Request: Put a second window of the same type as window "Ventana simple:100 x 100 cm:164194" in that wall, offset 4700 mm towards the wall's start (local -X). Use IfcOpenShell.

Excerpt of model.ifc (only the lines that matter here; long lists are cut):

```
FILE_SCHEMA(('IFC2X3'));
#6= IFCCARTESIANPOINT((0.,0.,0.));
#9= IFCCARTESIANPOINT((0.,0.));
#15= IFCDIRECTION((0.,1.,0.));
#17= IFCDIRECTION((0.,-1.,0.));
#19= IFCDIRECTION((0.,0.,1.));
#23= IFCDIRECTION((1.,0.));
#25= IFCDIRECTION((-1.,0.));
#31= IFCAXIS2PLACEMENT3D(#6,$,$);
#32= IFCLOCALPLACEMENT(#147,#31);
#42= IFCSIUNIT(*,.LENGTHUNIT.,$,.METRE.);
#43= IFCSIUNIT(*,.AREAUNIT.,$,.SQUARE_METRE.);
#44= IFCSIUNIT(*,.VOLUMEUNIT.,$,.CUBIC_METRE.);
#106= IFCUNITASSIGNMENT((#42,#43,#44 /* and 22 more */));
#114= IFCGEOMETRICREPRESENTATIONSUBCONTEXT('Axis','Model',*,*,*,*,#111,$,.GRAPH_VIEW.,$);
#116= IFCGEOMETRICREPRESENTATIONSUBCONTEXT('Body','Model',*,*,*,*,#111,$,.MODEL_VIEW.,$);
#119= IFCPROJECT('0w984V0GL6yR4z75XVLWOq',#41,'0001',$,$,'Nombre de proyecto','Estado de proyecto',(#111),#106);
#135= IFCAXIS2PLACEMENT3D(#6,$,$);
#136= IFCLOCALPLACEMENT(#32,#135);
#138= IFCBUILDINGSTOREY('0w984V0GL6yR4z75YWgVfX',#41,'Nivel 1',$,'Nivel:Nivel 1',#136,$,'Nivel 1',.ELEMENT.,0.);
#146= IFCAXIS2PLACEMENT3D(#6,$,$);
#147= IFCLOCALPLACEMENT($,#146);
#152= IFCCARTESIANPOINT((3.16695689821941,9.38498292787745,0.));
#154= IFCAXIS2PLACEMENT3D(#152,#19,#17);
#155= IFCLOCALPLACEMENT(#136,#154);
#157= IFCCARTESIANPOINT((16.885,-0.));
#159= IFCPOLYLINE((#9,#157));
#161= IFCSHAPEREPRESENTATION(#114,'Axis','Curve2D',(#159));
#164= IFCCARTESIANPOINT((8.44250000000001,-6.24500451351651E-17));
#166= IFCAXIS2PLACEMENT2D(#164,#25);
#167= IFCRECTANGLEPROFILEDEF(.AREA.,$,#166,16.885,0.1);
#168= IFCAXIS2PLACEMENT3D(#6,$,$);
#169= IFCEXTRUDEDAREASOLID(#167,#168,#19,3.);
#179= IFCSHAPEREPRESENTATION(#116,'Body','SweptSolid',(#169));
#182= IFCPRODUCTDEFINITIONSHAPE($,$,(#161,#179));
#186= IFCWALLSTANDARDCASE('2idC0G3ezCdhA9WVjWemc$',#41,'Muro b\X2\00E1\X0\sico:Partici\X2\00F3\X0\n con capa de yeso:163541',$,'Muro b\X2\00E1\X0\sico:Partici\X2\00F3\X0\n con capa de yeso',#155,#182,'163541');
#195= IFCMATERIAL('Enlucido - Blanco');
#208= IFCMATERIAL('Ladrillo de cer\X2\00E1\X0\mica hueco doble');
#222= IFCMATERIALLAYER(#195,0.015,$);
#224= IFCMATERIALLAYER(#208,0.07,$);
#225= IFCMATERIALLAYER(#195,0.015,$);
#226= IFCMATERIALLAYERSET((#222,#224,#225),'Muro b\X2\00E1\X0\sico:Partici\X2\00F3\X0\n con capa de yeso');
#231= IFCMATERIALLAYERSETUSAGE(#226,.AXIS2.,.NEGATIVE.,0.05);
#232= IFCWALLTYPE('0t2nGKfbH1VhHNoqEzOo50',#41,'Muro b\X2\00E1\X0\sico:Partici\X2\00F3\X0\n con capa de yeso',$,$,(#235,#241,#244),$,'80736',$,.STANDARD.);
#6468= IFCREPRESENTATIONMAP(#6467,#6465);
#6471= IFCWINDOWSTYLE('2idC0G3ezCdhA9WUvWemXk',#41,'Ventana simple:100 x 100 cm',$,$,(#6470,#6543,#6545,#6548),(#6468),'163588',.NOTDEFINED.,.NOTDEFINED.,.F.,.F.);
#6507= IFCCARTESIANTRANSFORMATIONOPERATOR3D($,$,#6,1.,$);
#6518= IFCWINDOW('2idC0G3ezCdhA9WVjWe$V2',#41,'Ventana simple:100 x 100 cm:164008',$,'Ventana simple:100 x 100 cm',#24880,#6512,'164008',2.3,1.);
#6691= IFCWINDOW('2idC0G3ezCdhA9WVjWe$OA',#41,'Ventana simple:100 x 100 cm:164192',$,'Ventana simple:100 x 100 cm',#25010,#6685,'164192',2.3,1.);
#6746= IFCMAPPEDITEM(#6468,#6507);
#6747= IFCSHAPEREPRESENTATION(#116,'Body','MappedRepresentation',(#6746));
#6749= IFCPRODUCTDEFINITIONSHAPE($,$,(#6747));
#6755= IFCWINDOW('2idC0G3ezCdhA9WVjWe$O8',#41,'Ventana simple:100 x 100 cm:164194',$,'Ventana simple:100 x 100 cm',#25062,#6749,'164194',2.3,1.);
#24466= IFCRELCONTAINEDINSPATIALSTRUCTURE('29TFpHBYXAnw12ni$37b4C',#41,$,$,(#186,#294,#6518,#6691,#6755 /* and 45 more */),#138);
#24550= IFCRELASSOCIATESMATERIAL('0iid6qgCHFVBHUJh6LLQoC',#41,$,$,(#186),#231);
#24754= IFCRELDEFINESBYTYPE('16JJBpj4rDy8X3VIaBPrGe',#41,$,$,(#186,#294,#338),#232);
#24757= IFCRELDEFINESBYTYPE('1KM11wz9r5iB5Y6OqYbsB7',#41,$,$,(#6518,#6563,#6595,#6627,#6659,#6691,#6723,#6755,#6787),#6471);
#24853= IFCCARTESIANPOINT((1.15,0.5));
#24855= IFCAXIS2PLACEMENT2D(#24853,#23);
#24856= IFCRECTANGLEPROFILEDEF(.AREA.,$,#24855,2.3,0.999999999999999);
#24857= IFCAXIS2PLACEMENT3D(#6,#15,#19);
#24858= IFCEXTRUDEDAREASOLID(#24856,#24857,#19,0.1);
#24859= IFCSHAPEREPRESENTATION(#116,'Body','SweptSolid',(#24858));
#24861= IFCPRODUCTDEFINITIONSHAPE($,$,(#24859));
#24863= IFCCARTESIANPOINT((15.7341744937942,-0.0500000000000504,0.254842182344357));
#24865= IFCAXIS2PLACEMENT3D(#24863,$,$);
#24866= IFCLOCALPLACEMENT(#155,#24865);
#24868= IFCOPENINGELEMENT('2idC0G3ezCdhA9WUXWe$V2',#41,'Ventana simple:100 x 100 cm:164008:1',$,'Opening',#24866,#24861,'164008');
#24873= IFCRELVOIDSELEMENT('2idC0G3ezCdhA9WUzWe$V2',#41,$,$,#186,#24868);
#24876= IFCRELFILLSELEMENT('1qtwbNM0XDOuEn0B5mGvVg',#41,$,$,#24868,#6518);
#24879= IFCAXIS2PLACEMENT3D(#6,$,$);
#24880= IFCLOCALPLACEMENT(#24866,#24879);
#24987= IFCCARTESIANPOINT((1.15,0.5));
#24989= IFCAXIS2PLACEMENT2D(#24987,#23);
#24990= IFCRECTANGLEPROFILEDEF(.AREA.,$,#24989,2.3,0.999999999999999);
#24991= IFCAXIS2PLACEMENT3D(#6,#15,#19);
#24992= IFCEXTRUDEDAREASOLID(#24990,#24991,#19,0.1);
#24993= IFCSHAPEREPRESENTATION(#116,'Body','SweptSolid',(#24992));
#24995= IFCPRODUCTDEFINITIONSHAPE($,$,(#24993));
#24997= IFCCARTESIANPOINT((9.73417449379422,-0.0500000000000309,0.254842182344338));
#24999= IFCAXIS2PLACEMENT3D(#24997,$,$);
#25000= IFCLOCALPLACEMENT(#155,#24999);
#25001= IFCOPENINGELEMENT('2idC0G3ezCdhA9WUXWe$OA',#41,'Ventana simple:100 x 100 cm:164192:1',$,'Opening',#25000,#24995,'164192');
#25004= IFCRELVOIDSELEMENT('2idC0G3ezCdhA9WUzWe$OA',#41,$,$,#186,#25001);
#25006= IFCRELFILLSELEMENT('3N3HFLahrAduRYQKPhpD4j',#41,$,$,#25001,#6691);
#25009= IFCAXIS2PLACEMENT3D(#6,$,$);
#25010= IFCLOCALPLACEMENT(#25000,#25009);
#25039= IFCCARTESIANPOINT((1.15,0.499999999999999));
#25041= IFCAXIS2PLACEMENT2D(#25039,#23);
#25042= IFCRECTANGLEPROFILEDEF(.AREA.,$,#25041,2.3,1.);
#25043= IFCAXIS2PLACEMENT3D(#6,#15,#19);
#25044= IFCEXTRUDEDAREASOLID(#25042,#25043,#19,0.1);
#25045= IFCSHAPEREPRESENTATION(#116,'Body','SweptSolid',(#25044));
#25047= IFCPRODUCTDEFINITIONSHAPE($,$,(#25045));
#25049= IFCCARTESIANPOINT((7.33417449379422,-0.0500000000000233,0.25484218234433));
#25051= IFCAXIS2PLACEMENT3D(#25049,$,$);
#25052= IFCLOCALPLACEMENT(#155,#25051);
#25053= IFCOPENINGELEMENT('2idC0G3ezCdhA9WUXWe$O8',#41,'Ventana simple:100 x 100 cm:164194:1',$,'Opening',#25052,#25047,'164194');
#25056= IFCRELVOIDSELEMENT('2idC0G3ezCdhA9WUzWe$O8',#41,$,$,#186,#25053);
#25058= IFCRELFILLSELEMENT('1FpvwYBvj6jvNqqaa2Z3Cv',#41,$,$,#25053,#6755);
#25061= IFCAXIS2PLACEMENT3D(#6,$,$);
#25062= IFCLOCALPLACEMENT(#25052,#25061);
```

```python
import ifcopenshell
import ifcopenshell.api.feature
import ifcopenshell.api.geometry
import ifcopenshell.api.root
import ifcopenshell.geom
import ifcopenshell.util.element
import ifcopenshell.util.placement
import ifcopenshell.util.shape
import ifcopenshell.util.unit

model = ifcopenshell.open("model.ifc")
unit_scale = ifcopenshell.util.unit.calculate_unit_scale(model)
settings = ifcopenshell.geom.settings()


def volume(element):
    """Net volume in cubic metres, openings subtracted."""
    shape = ifcopenshell.geom.create_shape(settings, element)
    return ifcopenshell.util.shape.get_volume(shape.geometry)


def reuse_history(source, copy):
    """copy_class also copies each property set's owner history, people and application; keep the originals."""
    for rel in copy.IsDefinedBy:
        if rel.is_a("IfcRelDefinesByProperties") and (history := rel.RelatingPropertyDefinition.OwnerHistory):
            rel.RelatingPropertyDefinition.OwnerHistory = source.OwnerHistory
            ifcopenshell.util.element.remove_deep2(model, history)


window = model.by_guid("2idC0G3ezCdhA9WVjWe$O8")
opening = window.FillsVoids[0].RelatingOpeningElement
wall = opening.VoidsElements[0].RelatingBuildingElement
before = volume(wall)
shift = ifcopenshell.util.placement.get_local_placement(wall.ObjectPlacement)[:3, 0] * -4.7 / unit_scale

# copy_class copies the void relationship, type, container and properties, but no geometry.
new_opening = ifcopenshell.api.root.copy_class(model, product=opening)
new_opening.Representation = ifcopenshell.util.element.copy_deep(
    model, opening.Representation, exclude=["IfcGeometricRepresentationContext", "IfcRepresentationMap"]
)
new_opening.Name = "Ventana simple:100 x 100 cm"
new_opening.Tag = None
new_window = ifcopenshell.api.root.copy_class(model, product=window)
new_window.Representation = ifcopenshell.util.element.copy_deep(
    model, window.Representation, exclude=["IfcGeometricRepresentationContext", "IfcRepresentationMap"]
)
new_window.Name = "Ventana simple:100 x 100 cm"
new_window.Tag = None
reuse_history(window, new_window)
fills = ifcopenshell.api.feature.add_filling(model, opening=new_opening, element=new_window)
fills.OwnerHistory = new_window.OwnerHistory  # required in IFC2X3

for old, new in ((opening, new_opening), (window, new_window)):
    matrix = ifcopenshell.util.placement.get_local_placement(old.ObjectPlacement)
    matrix[:3, 3] += shift
    ifcopenshell.api.geometry.edit_object_placement(model, product=new, matrix=matrix, is_si=False)

after = volume(wall)

print(f"wall volume {before:.3f} -> {after:.3f} m3")

model.write("model_updated.ifc")
```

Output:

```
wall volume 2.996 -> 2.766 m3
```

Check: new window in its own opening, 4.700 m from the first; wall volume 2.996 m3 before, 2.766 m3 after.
